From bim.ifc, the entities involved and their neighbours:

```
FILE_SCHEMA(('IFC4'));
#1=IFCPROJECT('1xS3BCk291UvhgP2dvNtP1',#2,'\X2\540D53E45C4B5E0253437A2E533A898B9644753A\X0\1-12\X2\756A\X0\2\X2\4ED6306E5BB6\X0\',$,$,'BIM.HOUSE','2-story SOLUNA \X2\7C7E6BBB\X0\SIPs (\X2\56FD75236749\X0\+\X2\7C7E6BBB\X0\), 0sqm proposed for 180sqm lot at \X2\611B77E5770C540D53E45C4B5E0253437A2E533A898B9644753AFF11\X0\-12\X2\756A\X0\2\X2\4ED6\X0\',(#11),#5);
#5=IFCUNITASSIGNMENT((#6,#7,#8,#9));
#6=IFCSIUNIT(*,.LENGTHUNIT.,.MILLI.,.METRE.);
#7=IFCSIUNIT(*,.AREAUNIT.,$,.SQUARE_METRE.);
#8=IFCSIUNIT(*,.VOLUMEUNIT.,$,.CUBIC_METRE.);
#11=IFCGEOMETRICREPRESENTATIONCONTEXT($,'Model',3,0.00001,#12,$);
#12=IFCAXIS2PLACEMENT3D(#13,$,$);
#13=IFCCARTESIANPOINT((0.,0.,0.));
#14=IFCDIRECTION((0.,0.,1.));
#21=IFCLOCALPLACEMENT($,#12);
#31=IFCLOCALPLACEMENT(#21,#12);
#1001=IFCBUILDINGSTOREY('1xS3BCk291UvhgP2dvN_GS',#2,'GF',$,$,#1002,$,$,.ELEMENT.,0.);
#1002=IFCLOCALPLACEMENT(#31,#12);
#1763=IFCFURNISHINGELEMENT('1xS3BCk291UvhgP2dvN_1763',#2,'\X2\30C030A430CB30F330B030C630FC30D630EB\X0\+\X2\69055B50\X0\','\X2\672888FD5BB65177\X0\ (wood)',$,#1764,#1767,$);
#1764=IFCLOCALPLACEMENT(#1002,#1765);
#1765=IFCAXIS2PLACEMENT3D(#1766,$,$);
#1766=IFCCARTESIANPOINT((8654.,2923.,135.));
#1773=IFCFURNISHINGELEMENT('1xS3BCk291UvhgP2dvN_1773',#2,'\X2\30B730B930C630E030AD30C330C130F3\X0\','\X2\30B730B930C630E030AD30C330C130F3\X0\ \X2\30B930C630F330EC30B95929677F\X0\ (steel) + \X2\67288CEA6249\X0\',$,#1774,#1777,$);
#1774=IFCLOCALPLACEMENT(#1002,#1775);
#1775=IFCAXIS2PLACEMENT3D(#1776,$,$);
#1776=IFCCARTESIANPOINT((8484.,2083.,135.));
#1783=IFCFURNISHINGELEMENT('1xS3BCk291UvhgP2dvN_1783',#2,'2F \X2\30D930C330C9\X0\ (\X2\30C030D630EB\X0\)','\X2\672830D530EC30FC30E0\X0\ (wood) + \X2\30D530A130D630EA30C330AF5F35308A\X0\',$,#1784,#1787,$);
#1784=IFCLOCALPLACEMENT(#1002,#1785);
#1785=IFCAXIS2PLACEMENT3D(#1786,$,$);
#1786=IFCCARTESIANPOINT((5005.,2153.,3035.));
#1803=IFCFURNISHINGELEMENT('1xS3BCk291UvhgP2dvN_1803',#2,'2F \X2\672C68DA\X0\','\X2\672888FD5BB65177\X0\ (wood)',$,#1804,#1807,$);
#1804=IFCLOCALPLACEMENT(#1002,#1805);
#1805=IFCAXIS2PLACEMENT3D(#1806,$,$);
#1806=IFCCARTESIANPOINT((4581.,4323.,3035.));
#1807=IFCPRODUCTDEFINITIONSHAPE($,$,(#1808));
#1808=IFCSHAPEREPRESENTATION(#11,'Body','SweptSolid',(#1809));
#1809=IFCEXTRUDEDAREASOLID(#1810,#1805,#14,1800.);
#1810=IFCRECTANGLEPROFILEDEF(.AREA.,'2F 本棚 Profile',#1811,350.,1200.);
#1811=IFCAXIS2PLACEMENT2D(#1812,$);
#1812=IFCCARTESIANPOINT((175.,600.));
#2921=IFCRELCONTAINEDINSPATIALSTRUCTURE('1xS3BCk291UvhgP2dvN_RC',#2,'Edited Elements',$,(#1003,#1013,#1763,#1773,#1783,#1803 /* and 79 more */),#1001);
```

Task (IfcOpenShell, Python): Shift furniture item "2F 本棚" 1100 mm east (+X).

```python
import ifcopenshell
import ifcopenshell.api.geometry
import ifcopenshell.util.placement
import ifcopenshell.util.unit

model = ifcopenshell.open("bim.ifc")
unit_scale = ifcopenshell.util.unit.calculate_unit_scale(model)

item = model.by_guid("1xS3BCk291UvhgP2dvN_1803")
matrix = ifcopenshell.util.placement.get_local_placement(item.ObjectPlacement)
matrix[0, 3] += 1.1 / unit_scale
ifcopenshell.api.geometry.edit_object_placement(model, product=item, matrix=matrix, is_si=False)

print(ifcopenshell.util.placement.get_local_placement(item.ObjectPlacement).round(3) + 0.0)

model.write("bim_edited.ifc")
```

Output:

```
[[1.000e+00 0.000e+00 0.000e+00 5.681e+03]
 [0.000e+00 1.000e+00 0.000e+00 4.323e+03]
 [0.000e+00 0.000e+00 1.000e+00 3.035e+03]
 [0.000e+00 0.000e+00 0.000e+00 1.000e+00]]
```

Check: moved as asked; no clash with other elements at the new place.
